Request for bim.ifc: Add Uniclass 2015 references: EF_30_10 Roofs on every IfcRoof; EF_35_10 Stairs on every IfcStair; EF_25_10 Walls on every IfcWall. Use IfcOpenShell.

First a look at what the model holds.

```python
import ifcopenshell

model = ifcopenshell.open("bim.ifc")
print(model.schema)
print("classifications:", [c.Name for c in model.by_type("IfcClassification")])
for ifc_class in ("IfcDoor", "IfcRoof", "IfcStair", "IfcWall", "IfcWindow"):
    print(ifc_class, len(model.by_type(ifc_class)))
```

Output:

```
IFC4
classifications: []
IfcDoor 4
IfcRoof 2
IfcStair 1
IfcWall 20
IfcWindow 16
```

```python
import ifcopenshell
import ifcopenshell.api.classification

model = ifcopenshell.open("bim.ifc")

system = ifcopenshell.api.classification.add_classification(model, classification="Uniclass 2015")

codes = {
    "IfcRoof": ("EF_30_10", "Roofs"),
    "IfcStair": ("EF_35_10", "Stairs"),
    "IfcWall": ("EF_25_10", "Walls"),
}
for ifc_class, (code, name) in codes.items():
    products = model.by_type(ifc_class)
    ifcopenshell.api.classification.add_reference(
        model, products=products, classification=system, identification=code, name=name
    )
    print(code, len(products))

model.write("bim_updated.ifc")
```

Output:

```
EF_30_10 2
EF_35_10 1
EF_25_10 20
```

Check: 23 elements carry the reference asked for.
